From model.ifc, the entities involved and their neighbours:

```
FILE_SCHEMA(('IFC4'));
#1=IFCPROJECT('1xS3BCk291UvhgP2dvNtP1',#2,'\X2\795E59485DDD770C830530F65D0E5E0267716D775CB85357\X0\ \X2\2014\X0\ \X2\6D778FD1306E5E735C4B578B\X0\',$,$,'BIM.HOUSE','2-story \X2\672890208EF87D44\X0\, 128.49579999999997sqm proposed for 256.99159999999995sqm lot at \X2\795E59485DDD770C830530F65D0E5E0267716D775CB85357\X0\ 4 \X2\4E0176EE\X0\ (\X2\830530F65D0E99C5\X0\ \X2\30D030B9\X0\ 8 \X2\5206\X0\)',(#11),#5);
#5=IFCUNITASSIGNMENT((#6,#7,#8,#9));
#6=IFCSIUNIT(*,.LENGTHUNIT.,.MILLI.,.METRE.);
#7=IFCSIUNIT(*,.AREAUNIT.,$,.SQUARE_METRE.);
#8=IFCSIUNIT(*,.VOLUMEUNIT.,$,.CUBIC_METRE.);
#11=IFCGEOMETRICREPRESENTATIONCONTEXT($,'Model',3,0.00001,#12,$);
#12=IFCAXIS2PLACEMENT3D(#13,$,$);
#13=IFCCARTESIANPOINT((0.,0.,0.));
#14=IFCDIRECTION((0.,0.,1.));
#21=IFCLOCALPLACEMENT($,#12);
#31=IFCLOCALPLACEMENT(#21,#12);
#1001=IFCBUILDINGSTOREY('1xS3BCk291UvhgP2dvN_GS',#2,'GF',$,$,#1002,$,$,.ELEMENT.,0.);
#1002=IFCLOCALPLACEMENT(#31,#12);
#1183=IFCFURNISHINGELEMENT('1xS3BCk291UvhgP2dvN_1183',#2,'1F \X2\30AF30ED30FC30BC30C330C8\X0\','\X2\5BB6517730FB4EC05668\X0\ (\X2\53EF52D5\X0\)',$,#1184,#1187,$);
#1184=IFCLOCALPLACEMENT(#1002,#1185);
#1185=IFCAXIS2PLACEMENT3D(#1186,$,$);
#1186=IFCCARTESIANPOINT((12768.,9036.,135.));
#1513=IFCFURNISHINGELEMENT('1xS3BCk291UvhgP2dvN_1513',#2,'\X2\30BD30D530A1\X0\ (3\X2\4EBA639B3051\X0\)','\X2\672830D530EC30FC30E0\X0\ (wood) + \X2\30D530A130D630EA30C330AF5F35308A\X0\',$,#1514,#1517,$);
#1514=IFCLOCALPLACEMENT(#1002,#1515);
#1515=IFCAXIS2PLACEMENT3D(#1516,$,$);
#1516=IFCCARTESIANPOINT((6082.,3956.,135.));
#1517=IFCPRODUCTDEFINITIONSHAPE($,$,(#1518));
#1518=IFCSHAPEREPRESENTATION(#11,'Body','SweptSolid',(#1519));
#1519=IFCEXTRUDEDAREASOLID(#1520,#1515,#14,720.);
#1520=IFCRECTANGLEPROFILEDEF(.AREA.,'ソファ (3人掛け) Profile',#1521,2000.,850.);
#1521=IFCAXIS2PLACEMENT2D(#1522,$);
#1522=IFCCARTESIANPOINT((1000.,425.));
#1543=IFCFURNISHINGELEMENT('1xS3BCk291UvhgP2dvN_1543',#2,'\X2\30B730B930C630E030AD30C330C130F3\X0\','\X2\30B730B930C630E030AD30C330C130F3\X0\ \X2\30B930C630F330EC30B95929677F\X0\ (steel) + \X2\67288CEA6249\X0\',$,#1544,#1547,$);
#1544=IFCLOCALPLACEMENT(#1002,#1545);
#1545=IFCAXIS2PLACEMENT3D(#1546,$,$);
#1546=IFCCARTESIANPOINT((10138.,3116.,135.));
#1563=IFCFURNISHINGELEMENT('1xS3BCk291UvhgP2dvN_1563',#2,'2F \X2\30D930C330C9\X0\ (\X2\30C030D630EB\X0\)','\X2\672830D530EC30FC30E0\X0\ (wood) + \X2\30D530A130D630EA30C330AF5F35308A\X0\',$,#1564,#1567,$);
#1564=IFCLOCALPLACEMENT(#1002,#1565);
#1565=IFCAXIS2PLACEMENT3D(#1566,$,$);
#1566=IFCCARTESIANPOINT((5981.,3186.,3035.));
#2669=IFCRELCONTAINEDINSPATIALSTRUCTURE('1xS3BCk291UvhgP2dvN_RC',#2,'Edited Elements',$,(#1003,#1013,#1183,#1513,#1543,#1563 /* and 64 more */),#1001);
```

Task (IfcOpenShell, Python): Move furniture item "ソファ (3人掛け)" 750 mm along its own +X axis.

```python
import ifcopenshell
import ifcopenshell.api.geometry
import ifcopenshell.util.placement

model = ifcopenshell.open("model.ifc")

item = model.by_id(1513)
matrix = ifcopenshell.util.placement.get_local_placement(item.ObjectPlacement)
matrix[:3, 3] += matrix[:3, 0] * 750.0
ifcopenshell.api.geometry.edit_object_placement(model, product=item, matrix=matrix, is_si=False)

print(ifcopenshell.util.placement.get_local_placement(item.ObjectPlacement).round(3) + 0.0)

model.write("model_edited.ifc")
```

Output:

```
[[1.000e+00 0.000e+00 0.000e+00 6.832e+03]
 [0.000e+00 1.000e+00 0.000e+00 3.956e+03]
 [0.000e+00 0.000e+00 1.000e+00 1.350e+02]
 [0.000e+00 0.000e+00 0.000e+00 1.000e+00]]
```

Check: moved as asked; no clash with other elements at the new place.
